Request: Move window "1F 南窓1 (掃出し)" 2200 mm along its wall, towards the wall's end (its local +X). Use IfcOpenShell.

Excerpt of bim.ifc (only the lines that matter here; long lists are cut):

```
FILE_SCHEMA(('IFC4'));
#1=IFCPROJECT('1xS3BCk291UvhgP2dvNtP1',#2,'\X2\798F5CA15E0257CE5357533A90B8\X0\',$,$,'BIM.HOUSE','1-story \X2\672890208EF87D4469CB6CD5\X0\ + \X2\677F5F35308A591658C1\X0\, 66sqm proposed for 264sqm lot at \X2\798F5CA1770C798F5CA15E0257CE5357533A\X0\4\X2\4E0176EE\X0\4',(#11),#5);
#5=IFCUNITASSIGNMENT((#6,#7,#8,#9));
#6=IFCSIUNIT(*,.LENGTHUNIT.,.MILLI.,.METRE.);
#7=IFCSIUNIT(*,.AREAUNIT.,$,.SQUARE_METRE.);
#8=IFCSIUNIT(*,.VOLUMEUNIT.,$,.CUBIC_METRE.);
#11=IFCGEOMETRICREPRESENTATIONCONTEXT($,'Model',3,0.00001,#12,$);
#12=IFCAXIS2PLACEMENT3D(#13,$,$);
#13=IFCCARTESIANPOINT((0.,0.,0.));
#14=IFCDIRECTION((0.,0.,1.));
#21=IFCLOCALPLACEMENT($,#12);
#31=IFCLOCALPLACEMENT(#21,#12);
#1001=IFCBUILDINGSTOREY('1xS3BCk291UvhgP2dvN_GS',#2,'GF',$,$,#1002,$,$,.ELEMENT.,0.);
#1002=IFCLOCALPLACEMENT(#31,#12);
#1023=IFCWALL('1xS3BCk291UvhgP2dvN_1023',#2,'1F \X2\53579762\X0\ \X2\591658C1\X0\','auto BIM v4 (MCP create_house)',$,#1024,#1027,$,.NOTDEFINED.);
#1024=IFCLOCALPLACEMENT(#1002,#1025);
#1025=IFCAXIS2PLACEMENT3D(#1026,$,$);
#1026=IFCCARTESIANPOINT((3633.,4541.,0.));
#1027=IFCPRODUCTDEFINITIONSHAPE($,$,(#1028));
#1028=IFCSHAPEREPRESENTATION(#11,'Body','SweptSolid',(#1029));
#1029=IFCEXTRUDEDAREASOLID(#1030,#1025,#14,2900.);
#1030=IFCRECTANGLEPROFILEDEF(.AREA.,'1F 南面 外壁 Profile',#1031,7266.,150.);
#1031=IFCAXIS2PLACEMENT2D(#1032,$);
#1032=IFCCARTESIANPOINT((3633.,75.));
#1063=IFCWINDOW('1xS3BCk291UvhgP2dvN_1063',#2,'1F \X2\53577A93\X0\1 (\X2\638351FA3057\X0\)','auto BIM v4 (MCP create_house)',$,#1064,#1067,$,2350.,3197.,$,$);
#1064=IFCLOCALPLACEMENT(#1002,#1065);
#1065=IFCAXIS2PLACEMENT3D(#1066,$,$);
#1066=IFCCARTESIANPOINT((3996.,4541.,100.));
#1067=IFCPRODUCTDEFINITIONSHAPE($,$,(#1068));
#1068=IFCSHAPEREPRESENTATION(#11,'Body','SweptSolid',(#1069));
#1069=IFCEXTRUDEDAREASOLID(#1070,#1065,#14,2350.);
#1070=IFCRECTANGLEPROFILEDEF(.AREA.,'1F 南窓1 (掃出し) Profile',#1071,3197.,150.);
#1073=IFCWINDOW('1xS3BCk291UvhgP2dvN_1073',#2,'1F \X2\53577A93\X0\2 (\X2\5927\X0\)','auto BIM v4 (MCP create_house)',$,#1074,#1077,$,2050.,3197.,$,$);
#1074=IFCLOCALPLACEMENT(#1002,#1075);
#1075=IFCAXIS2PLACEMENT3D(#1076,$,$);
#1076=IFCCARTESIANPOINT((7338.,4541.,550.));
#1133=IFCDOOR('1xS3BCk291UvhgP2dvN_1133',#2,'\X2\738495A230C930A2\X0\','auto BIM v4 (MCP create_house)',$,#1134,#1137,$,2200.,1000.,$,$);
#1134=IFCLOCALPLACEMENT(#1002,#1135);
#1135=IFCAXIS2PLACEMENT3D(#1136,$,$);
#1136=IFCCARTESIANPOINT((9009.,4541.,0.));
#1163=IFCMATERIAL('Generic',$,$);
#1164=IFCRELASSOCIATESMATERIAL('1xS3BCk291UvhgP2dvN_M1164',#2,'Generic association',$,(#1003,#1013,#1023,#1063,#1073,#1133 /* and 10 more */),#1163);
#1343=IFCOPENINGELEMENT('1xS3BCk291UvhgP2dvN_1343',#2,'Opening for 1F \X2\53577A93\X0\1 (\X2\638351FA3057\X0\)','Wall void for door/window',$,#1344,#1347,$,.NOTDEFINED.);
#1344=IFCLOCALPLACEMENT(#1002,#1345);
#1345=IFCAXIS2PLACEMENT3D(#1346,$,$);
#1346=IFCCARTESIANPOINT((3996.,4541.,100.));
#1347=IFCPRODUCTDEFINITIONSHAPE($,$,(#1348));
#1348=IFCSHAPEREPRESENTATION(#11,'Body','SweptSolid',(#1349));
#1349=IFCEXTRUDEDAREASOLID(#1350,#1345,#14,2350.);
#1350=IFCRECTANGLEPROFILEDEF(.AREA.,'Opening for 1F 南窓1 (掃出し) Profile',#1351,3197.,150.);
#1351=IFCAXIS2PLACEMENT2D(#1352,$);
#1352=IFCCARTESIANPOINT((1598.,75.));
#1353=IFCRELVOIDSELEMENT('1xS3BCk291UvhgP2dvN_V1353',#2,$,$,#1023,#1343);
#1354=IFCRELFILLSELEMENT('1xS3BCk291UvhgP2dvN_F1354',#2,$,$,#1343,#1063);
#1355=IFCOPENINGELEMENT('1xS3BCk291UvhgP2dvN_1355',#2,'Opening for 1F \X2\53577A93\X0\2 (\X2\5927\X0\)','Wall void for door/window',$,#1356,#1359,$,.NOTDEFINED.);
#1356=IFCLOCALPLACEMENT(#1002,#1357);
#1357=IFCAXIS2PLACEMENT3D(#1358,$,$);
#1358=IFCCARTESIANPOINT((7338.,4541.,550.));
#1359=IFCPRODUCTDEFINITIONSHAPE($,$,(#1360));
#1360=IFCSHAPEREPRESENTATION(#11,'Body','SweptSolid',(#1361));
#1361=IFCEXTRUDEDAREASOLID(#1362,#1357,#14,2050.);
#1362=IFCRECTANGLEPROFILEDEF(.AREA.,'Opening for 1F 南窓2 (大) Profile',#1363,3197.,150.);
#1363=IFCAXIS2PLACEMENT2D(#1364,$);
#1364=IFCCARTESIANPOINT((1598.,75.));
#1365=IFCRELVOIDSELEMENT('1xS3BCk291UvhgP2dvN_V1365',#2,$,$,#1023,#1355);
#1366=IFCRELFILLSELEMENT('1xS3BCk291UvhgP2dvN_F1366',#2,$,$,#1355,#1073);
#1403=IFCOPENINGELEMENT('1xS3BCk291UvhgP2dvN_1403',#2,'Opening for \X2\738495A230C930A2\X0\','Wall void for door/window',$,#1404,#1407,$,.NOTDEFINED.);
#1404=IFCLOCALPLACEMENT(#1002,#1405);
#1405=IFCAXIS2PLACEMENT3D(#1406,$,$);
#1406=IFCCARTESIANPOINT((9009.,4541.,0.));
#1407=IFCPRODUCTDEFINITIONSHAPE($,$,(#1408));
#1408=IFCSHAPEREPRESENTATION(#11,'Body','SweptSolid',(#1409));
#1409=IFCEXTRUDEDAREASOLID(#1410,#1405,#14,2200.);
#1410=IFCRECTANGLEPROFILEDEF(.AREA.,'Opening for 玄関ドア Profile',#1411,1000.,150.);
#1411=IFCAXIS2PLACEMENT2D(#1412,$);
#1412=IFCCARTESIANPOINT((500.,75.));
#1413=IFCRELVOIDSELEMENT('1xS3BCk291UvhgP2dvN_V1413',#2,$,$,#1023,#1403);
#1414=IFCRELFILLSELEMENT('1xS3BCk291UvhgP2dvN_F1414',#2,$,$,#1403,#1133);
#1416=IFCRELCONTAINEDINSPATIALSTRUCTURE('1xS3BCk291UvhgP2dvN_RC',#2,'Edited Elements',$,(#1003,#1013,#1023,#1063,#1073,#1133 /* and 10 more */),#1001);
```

```python
import ifcopenshell
import ifcopenshell.api.geometry
import ifcopenshell.util.placement

model = ifcopenshell.open("bim.ifc")

window = model.by_guid("1xS3BCk291UvhgP2dvN_1063")
opening = window.FillsVoids[0].RelatingOpeningElement
wall = opening.VoidsElements[0].RelatingBuildingElement

wall_matrix = ifcopenshell.util.placement.get_local_placement(wall.ObjectPlacement)
shift = wall_matrix[:3, 0] * 2200.0
before = ifcopenshell.util.placement.get_local_placement(window.ObjectPlacement)[:3, 3].copy()

# The window is not placed relative to its opening, so move both.
for product in (opening, window):
    matrix = ifcopenshell.util.placement.get_local_placement(product.ObjectPlacement)
    matrix[:3, 3] += shift
    ifcopenshell.api.geometry.edit_object_placement(model, product=product, matrix=matrix, is_si=False)

after = ifcopenshell.util.placement.get_local_placement(window.ObjectPlacement)[:3, 3]
print("window moved by", (after - before).round(3) + 0.0)

model.write("bim_updated.ifc")
```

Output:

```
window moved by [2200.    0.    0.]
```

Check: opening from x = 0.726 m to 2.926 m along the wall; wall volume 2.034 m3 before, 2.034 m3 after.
